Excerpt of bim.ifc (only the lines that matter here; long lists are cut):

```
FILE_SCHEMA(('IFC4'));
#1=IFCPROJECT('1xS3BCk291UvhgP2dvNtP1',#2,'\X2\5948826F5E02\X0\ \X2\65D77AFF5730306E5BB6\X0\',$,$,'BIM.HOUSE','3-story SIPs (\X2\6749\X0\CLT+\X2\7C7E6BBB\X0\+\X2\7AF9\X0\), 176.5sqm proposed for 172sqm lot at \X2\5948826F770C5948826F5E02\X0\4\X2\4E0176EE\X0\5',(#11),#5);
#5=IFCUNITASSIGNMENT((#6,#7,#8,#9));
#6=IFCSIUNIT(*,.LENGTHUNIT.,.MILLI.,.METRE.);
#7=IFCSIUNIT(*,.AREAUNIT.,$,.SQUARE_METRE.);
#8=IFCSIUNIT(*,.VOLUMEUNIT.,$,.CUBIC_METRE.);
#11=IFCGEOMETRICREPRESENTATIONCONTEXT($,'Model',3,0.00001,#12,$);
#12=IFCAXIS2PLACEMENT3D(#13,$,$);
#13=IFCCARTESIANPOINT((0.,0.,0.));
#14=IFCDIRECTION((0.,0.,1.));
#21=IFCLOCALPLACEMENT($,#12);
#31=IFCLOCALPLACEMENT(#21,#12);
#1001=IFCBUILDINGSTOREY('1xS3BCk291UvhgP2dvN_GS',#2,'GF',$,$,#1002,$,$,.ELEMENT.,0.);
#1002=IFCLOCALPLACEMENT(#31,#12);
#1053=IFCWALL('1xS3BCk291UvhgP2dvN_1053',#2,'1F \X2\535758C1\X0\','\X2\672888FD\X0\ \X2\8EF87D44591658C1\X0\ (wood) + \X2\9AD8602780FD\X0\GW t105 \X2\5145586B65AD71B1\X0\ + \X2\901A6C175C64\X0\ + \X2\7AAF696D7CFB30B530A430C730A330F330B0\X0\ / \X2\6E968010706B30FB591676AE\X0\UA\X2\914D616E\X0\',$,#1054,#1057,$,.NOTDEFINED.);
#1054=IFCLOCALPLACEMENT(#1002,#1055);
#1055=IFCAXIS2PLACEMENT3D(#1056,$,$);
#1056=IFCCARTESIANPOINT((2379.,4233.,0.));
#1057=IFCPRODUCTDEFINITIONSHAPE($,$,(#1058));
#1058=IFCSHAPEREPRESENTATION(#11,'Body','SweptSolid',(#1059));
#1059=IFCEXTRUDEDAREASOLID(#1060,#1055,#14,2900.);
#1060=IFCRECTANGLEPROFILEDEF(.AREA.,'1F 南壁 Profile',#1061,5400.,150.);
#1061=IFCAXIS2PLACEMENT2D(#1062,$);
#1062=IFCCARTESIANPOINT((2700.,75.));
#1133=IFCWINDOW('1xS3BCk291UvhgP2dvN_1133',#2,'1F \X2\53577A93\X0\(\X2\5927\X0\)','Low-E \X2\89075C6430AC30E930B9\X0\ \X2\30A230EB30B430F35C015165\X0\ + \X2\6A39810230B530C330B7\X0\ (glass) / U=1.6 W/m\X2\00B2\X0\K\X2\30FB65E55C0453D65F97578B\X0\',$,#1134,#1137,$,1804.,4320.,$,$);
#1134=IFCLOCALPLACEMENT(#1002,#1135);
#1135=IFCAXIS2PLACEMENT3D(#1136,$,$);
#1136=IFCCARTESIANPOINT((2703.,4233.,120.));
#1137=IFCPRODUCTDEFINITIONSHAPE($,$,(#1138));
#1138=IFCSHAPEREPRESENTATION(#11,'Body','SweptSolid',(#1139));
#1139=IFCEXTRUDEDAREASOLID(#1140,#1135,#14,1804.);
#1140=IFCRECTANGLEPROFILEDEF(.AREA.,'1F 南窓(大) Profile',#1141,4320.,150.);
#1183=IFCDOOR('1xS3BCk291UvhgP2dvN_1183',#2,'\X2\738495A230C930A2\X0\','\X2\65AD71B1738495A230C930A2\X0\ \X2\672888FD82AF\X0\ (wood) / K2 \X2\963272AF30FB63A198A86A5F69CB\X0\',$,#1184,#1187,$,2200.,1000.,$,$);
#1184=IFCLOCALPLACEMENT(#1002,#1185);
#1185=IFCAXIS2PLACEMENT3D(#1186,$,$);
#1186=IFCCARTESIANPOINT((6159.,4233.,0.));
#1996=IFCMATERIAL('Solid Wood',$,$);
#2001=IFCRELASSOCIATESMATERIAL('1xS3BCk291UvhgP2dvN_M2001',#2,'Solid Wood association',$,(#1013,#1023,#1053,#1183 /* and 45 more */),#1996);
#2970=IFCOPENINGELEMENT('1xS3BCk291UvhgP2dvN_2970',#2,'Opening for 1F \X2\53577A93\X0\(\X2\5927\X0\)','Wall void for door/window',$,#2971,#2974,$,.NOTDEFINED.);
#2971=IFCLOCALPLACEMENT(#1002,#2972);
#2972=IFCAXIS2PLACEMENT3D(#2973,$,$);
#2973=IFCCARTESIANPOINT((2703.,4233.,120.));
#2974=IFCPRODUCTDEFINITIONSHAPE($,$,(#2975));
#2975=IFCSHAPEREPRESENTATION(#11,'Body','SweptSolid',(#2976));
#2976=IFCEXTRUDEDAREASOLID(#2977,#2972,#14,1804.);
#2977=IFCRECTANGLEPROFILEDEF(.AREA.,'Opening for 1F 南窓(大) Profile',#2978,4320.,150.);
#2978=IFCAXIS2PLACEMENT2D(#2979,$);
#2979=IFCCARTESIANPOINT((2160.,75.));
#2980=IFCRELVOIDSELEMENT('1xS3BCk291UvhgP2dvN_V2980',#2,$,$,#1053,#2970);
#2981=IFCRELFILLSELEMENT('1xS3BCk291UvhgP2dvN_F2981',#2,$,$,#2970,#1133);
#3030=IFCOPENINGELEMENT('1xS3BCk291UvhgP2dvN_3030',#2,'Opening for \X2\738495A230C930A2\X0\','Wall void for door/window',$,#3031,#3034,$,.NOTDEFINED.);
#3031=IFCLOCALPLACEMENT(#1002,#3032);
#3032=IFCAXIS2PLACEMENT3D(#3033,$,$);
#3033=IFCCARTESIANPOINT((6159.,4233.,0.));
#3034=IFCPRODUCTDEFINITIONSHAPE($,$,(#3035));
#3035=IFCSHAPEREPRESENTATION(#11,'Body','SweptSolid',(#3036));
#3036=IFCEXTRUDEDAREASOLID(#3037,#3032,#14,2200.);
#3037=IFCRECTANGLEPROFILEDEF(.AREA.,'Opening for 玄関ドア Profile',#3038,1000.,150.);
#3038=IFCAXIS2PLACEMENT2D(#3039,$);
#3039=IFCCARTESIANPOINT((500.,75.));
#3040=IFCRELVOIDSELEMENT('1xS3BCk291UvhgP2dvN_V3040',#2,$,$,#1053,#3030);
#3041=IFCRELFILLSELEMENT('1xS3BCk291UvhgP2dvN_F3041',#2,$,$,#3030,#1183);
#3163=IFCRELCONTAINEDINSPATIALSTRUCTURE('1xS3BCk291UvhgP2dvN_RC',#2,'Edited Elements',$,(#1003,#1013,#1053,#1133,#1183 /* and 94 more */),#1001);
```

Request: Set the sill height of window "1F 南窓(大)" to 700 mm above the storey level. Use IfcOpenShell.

```python
import numpy as np
import ifcopenshell
import ifcopenshell.api.geometry
import ifcopenshell.geom
import ifcopenshell.util.element
import ifcopenshell.util.placement
import ifcopenshell.util.shape
import ifcopenshell.util.unit

model = ifcopenshell.open("bim.ifc")
unit_scale = ifcopenshell.util.unit.calculate_unit_scale(model)

window = model.by_guid("1xS3BCk291UvhgP2dvN_1133")
opening = window.FillsVoids[0].RelatingOpeningElement
storey = ifcopenshell.util.element.get_container(window, ifc_class="IfcBuildingStorey")
level = ifcopenshell.util.placement.get_local_placement(storey.ObjectPlacement)[2, 3]

# The opening's origin need not be at the sill, so measure its lowest point.
shape = ifcopenshell.geom.create_shape(ifcopenshell.geom.settings(), opening)
bottom = ifcopenshell.util.shape.get_shape_bottom_elevation(shape, shape.geometry) / unit_scale
dz = level + 700.0 - bottom

shift = np.array([0.0, 0.0, dz])
# The window is not placed relative to its opening, so move both.
for product in (opening, window):
    matrix = ifcopenshell.util.placement.get_local_placement(product.ObjectPlacement)
    matrix[:3, 3] += shift
    ifcopenshell.api.geometry.edit_object_placement(model, product=product, matrix=matrix, is_si=False)

print(f"moved by {dz * unit_scale:+.3f} m")

model.write("bim_updated.ifc")
```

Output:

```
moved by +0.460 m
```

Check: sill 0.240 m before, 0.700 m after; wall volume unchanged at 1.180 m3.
